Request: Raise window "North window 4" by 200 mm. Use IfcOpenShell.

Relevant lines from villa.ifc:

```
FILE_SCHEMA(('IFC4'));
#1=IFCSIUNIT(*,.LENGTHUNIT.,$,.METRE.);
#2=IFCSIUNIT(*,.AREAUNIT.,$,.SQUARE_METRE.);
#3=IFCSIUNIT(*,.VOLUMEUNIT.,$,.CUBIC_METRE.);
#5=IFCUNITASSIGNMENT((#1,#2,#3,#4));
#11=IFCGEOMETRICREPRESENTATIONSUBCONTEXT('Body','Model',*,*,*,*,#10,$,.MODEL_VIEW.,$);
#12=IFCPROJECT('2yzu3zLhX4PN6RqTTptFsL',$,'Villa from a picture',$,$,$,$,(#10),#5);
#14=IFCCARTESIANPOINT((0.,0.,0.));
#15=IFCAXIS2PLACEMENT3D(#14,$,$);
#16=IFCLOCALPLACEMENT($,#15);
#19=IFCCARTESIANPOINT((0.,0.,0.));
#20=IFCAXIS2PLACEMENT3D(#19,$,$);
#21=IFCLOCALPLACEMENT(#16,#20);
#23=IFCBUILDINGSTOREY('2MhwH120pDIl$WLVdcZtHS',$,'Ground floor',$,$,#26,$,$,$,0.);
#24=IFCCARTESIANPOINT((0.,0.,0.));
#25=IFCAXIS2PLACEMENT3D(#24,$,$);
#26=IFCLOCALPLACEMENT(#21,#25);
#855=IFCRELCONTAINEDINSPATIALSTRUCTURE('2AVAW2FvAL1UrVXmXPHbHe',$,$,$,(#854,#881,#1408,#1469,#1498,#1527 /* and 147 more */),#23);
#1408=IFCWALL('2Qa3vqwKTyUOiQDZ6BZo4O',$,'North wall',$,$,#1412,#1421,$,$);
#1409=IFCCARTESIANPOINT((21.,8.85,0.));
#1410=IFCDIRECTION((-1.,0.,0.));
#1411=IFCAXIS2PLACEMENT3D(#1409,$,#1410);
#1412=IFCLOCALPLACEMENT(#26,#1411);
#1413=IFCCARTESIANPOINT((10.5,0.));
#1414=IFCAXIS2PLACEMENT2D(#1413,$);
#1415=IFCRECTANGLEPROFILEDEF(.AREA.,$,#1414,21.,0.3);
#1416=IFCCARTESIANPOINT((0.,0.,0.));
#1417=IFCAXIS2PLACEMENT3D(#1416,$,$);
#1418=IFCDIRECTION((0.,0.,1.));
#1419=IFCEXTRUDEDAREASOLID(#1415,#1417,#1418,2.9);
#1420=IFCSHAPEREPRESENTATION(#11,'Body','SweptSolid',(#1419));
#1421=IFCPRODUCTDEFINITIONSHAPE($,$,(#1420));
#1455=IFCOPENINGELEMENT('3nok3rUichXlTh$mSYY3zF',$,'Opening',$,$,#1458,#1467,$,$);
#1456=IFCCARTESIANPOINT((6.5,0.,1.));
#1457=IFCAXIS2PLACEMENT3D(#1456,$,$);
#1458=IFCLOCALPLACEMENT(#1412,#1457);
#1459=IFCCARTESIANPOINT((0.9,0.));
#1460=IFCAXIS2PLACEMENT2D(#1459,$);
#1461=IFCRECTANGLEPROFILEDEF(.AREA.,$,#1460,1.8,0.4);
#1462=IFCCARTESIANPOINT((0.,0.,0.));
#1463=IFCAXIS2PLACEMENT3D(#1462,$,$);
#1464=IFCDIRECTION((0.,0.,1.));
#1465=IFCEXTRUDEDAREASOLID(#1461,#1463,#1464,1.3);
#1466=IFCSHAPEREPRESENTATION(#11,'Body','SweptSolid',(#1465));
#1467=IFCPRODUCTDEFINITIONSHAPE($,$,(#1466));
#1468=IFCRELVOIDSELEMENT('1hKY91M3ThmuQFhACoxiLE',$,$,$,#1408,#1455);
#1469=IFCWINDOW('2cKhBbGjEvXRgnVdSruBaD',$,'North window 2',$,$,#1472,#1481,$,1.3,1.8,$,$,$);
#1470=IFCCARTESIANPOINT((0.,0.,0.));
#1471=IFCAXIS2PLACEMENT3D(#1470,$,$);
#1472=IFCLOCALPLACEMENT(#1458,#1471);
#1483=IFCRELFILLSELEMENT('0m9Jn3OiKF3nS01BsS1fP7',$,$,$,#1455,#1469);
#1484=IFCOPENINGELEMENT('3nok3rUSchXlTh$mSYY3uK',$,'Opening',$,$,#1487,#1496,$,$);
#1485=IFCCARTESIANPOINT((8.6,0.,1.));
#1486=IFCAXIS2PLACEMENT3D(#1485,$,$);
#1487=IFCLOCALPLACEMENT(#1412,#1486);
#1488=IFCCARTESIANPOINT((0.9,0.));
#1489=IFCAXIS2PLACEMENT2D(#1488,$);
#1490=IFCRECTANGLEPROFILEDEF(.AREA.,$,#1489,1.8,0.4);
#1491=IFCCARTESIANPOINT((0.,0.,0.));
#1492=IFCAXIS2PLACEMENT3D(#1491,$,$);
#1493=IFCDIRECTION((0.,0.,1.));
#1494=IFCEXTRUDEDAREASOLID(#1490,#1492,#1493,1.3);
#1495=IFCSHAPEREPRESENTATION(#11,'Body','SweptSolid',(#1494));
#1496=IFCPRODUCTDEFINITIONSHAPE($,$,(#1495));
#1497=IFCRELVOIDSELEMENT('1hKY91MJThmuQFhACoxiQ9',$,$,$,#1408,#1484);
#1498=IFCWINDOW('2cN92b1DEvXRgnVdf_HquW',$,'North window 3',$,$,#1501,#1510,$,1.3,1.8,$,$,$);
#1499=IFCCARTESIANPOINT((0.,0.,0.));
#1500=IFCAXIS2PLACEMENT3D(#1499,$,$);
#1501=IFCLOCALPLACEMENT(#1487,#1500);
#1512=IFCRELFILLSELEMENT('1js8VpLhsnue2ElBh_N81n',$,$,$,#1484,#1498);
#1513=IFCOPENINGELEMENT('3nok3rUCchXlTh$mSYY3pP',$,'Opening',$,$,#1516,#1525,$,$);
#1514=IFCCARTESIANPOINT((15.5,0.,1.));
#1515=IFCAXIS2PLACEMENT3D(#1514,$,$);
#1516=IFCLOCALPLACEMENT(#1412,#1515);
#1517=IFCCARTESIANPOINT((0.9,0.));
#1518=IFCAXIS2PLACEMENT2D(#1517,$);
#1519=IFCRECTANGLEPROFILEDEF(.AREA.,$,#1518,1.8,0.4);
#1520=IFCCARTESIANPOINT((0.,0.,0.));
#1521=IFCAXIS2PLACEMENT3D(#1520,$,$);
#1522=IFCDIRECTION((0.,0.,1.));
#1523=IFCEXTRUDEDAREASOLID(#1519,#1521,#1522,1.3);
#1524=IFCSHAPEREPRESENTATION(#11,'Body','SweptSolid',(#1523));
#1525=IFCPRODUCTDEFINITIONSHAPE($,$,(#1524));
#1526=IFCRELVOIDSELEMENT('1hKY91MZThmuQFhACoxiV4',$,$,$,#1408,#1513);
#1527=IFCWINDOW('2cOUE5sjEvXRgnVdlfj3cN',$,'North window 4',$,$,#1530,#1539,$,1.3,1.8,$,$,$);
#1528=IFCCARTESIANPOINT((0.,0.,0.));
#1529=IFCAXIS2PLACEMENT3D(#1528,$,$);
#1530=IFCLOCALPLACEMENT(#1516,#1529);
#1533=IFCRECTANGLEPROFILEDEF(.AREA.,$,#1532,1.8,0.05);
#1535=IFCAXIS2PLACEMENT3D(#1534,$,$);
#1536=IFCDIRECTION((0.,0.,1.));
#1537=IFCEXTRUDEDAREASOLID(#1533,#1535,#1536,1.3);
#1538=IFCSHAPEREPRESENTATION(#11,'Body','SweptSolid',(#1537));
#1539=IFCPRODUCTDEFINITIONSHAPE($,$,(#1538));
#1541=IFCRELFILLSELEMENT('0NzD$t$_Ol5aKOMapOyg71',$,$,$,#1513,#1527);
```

```python
import numpy as np
import ifcopenshell
import ifcopenshell.api.geometry
import ifcopenshell.util.placement
import ifcopenshell.util.unit

model = ifcopenshell.open("villa.ifc")
unit_scale = ifcopenshell.util.unit.calculate_unit_scale(model)

window = model.by_id(1527)
opening = window.FillsVoids[0].RelatingOpeningElement
dz = 0.2

shift = np.array([0.0, 0.0, dz])
# The window is placed relative to its opening, so it follows when the opening moves.
matrix = ifcopenshell.util.placement.get_local_placement(opening.ObjectPlacement)
matrix[:3, 3] += shift
ifcopenshell.api.geometry.edit_object_placement(
    model, product=opening, matrix=matrix, is_si=False, should_transform_children=True
)

print(f"moved by {dz * unit_scale:+.3f} m")

model.write("villa_rev.ifc")
```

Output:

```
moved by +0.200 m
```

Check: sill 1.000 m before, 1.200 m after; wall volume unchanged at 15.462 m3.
